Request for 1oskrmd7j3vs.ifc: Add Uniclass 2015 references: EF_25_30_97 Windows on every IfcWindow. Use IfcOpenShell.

First a look at what the model holds.

```python
import ifcopenshell

model = ifcopenshell.open("1oskrmd7j3vs.ifc")
print(model.schema)
print("classifications:", [c.Name for c in model.by_type("IfcClassification")])
for ifc_class in ("IfcDoor", "IfcRoof", "IfcStair", "IfcWall", "IfcWindow"):
    print(ifc_class, len(model.by_type(ifc_class)))
```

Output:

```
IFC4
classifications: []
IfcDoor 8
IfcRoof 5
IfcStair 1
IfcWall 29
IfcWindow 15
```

```python
import ifcopenshell
import ifcopenshell.api.classification

model = ifcopenshell.open("1oskrmd7j3vs.ifc")

system = ifcopenshell.api.classification.add_classification(model, classification="Uniclass 2015")

codes = {
    "IfcWindow": ("EF_25_30_97", "Windows"),
}
for ifc_class, (code, name) in codes.items():
    products = model.by_type(ifc_class)
    ifcopenshell.api.classification.add_reference(
        model, products=products, classification=system, identification=code, name=name
    )
    print(code, len(products))

model.write("1oskrmd7j3vs_updated.ifc")
```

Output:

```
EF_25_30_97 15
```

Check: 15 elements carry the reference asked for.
